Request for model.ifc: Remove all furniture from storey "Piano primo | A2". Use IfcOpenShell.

First a look at what the model holds.

```python
import ifcopenshell
import ifcopenshell.util.element

model = ifcopenshell.open("model.ifc")
print(model.schema)
storey = next(s for s in model.by_type("IfcBuildingStorey") if s.Name == "Piano primo | A2")
furniture = [e for e in ifcopenshell.util.element.get_decomposition(storey) if e.is_a("IfcFurnishingElement")]
seen = {}
for e in furniture:
    element_type = ifcopenshell.util.element.get_type(e)
    name = element_type.Name if element_type not in (None, e) else None
    seen[name] = seen.get(name, 0) + 1
for name, count in sorted(seen.items(), key=str):
    print(count, "x", name)
```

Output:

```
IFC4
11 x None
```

```python
import ifcopenshell
import ifcopenshell.api.root
import ifcopenshell.util.element

model = ifcopenshell.open("model.ifc")

storey = next(s for s in model.by_type("IfcBuildingStorey") if s.Name == "Piano primo | A2")
furniture = [e for e in ifcopenshell.util.element.get_decomposition(storey) if e.is_a("IfcFurnishingElement")]

for e in furniture:
    ifcopenshell.api.root.remove_product(model, product=e)
print(len(furniture), "removed")

model.write("model_rev.ifc")
```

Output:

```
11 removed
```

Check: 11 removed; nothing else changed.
